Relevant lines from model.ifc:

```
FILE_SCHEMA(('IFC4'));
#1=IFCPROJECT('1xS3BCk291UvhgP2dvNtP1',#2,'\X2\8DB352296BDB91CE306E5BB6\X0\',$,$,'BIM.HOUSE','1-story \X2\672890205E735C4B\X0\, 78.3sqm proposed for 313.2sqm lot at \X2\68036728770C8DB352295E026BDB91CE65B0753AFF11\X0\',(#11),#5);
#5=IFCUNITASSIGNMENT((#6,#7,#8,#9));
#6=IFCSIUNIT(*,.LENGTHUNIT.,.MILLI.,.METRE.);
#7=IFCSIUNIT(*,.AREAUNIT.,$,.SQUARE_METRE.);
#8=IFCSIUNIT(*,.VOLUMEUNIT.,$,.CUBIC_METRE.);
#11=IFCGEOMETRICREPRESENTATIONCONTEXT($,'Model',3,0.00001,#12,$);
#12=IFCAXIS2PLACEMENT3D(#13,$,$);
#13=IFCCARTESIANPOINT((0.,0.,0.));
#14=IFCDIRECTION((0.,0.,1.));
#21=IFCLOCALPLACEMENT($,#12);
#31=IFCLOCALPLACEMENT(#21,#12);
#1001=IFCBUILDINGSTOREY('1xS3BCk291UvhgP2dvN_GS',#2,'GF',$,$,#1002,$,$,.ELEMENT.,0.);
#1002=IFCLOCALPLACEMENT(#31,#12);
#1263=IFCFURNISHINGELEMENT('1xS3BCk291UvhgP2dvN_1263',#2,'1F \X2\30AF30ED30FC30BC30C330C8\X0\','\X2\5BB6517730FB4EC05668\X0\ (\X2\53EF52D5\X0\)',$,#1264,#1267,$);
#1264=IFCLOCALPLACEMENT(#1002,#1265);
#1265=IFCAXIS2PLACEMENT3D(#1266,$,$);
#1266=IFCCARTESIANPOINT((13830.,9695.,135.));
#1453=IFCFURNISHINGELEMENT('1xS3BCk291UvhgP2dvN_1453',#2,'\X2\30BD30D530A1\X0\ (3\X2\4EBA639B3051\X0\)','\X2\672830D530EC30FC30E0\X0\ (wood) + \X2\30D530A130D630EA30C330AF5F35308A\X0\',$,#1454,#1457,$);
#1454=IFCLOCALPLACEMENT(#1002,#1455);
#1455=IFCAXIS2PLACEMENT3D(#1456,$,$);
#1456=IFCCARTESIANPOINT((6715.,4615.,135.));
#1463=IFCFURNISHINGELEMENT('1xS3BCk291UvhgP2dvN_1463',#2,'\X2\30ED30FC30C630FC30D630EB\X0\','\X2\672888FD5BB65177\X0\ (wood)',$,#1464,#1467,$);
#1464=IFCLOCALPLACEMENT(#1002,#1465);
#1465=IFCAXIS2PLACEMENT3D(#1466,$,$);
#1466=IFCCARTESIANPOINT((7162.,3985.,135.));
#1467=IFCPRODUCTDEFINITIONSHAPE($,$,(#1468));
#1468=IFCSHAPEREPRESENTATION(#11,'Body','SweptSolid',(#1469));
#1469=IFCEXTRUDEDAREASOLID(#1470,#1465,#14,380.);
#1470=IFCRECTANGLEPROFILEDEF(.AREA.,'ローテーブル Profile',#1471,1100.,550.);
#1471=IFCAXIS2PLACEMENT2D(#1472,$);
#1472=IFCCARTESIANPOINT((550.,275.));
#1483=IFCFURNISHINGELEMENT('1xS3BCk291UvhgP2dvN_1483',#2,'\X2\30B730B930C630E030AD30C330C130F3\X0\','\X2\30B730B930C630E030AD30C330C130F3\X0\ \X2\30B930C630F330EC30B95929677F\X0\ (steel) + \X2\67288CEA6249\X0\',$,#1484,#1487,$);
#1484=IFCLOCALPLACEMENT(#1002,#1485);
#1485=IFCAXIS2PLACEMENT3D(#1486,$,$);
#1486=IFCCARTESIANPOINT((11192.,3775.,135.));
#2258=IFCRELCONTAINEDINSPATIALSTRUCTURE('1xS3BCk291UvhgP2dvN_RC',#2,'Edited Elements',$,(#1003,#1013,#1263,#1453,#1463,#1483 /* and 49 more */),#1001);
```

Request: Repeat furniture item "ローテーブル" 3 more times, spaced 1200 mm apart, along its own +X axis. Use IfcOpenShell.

```python
import ifcopenshell
import ifcopenshell.api.geometry
import ifcopenshell.api.root
import ifcopenshell.util.element
import ifcopenshell.util.placement
import ifcopenshell.util.unit

model = ifcopenshell.open("model.ifc")
unit_scale = ifcopenshell.util.unit.calculate_unit_scale(model)


def reuse_history(source, copy):
    """copy_class also copies each property set's owner history, people and application; keep the originals."""
    for rel in copy.IsDefinedBy:
        if rel.is_a("IfcRelDefinesByProperties") and (history := rel.RelatingPropertyDefinition.OwnerHistory):
            rel.RelatingPropertyDefinition.OwnerHistory = source.OwnerHistory
            ifcopenshell.util.element.remove_deep2(model, history)


source = model.by_guid("1xS3BCk291UvhgP2dvN_1463")
base = ifcopenshell.util.placement.get_local_placement(source.ObjectPlacement)
step = base[:3, 0] * 1.2 / unit_scale

for i in range(1, 4):
    copy = ifcopenshell.api.root.copy_class(model, product=source)
    copy.Representation = ifcopenshell.util.element.copy_deep(
        model, source.Representation, exclude=["IfcGeometricRepresentationContext", "IfcRepresentationMap"]
    )
    reuse_history(source, copy)
    matrix = base.copy()
    matrix[:3, 3] += i * step
    print("added at", matrix[:3, 3].round(3) + 0.0)
    ifcopenshell.api.geometry.edit_object_placement(model, product=copy, matrix=matrix, is_si=False)

model.write("model-out.ifc")
```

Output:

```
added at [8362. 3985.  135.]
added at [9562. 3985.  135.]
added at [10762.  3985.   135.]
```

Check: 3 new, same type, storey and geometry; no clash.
